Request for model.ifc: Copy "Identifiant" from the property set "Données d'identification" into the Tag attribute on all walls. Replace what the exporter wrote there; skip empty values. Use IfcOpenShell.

First a look at what the model holds.

```python
import ifcopenshell
import ifcopenshell.util.element

model = ifcopenshell.open("model.ifc")
print(model.schema)
walls = model.by_type("IfcWall")
print(len(walls), "walls")
for e in walls[:8]:
    source = ifcopenshell.util.element.get_pset(e, "Données d'identification", "Identifiant")
    target = e.Tag
    print(e.id(), repr(source), repr(target), sep=" | ")
```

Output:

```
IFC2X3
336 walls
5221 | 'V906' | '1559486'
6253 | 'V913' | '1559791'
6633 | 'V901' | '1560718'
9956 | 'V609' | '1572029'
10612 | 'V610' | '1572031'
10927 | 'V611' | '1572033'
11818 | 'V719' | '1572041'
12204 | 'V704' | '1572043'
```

```python
import ifcopenshell
import ifcopenshell.util.element

model = ifcopenshell.open("model.ifc")

count = 0
for e in model.by_type("IfcWall"):
    value = ifcopenshell.util.element.get_pset(e, "Données d'identification", "Identifiant")
    current = e.Tag
    if not value or not value.strip() or current == value:
        continue
    e.Tag = value
    count += 1

print(count, "walls updated")

model.write("model_rev.ifc")
```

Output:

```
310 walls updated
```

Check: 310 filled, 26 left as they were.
